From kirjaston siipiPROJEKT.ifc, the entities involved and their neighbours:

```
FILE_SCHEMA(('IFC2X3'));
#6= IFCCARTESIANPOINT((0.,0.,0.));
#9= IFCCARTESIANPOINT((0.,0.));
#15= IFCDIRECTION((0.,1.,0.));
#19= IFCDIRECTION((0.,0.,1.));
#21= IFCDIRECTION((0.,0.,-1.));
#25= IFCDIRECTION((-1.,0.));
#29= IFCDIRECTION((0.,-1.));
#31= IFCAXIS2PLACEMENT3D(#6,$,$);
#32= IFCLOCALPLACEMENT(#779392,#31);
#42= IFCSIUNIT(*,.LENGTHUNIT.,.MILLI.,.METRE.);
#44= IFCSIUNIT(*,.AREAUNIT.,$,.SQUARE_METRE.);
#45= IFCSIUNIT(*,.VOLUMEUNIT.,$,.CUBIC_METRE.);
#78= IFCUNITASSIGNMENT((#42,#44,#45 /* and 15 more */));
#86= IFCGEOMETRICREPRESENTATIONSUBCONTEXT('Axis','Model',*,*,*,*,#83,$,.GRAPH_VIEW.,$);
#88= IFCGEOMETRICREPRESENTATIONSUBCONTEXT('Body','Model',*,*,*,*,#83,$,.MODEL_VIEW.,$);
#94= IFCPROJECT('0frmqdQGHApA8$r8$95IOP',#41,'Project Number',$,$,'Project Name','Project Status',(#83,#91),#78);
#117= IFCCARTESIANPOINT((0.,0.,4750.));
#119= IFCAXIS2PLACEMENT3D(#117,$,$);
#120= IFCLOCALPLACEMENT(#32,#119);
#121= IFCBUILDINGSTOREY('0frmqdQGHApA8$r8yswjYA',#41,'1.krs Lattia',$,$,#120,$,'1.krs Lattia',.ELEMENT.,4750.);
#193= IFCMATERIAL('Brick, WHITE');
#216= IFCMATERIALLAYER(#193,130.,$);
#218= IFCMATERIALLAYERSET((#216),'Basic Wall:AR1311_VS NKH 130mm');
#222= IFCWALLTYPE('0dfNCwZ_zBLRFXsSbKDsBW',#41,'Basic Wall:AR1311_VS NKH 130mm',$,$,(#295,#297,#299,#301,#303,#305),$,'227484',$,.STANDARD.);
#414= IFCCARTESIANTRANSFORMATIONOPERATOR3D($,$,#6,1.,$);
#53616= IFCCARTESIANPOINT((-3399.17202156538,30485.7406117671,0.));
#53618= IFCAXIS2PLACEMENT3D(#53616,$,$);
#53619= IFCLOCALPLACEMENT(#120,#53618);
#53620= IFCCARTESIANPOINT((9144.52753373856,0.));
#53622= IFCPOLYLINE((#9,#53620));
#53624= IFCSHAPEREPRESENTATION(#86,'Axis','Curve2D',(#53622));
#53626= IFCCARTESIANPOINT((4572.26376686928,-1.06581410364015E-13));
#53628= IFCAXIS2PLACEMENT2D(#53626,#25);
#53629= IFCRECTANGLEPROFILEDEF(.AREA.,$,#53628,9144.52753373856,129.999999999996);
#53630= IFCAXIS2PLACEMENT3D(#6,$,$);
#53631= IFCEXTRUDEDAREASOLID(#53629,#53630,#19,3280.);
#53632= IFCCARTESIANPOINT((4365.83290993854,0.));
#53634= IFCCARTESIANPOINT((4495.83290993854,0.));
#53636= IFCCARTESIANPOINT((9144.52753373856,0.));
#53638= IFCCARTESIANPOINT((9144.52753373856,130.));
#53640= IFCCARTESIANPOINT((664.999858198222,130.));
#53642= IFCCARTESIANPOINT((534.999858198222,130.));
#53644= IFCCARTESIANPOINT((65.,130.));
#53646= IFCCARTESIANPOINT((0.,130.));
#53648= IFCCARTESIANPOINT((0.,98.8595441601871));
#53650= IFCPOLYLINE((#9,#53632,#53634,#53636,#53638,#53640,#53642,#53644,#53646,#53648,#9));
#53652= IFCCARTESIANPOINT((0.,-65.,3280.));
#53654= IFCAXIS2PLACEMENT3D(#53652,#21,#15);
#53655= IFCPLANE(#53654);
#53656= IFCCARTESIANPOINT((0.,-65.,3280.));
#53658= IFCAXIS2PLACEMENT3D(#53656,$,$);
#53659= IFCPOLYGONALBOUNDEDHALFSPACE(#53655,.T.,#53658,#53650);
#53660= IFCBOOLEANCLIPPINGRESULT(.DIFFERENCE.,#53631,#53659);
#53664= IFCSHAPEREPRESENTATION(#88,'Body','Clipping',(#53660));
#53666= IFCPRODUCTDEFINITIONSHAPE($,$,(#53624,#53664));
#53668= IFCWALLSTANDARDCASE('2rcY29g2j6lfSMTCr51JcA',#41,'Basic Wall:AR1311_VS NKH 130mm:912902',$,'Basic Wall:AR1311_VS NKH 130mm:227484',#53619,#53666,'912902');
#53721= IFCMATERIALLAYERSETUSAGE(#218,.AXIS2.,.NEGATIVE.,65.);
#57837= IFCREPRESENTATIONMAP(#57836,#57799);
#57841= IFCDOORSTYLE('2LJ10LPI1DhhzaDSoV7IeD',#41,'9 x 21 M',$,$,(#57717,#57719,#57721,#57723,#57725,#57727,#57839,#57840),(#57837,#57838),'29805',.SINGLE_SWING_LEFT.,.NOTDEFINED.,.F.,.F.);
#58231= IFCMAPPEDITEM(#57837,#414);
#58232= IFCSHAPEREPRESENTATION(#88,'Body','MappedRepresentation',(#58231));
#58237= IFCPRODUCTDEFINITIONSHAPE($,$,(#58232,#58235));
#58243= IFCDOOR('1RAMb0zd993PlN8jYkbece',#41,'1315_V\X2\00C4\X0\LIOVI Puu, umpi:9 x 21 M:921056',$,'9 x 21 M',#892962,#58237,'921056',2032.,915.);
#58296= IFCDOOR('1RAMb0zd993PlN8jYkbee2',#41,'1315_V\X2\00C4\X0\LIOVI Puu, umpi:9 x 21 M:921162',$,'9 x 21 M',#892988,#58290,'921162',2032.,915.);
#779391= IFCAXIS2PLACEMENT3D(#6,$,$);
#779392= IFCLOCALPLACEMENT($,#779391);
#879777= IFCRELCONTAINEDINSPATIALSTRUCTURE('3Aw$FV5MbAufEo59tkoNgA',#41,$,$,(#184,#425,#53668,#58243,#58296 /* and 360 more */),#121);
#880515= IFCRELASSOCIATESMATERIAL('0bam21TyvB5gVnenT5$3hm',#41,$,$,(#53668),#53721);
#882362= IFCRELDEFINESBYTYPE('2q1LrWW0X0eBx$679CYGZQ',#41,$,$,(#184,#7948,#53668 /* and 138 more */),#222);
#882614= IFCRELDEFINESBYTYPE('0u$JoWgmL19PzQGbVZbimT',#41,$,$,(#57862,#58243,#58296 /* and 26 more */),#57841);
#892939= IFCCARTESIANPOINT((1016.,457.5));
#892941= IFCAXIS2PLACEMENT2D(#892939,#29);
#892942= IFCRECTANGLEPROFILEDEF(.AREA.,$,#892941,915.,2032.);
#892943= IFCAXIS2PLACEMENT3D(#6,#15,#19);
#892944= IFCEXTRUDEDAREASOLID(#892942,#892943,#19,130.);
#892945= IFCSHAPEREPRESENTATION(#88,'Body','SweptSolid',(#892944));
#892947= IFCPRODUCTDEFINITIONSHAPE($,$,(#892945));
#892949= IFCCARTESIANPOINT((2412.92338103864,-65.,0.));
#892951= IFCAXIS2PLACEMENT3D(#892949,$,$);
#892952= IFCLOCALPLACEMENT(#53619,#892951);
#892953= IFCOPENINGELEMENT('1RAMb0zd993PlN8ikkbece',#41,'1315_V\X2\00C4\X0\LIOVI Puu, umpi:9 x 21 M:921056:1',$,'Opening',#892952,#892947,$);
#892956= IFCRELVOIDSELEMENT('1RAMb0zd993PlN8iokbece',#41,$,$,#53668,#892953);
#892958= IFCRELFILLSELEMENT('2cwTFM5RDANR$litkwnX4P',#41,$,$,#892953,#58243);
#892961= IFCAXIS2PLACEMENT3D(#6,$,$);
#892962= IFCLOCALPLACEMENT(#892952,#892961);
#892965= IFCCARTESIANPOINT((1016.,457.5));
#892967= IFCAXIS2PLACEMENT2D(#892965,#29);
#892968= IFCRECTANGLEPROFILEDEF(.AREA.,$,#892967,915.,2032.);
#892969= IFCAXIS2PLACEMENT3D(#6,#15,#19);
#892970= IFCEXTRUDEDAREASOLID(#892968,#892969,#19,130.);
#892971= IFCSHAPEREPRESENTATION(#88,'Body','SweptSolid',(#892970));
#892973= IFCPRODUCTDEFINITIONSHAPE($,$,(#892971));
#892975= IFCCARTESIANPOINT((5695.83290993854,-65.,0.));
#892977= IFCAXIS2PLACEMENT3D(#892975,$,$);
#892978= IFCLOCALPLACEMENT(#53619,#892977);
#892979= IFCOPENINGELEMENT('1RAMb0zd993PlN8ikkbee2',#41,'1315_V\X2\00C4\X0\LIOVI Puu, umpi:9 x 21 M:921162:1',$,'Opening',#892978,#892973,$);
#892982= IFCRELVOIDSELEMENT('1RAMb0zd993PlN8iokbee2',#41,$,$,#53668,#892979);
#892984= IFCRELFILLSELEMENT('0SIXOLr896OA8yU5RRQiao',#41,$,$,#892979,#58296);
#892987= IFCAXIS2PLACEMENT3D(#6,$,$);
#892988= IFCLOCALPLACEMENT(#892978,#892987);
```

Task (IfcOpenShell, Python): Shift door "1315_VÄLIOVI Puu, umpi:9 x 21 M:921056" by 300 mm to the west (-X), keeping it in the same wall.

```python
import ifcopenshell
import ifcopenshell.api.geometry
import ifcopenshell.util.placement

model = ifcopenshell.open("kirjaston siipiPROJEKT.ifc")

door = model.by_guid("1RAMb0zd993PlN8jYkbece")
opening = door.FillsVoids[0].RelatingOpeningElement
wall = opening.VoidsElements[0].RelatingBuildingElement

wall_matrix = ifcopenshell.util.placement.get_local_placement(wall.ObjectPlacement)
shift = wall_matrix[:3, 0] * -300.0
before = ifcopenshell.util.placement.get_local_placement(door.ObjectPlacement)[:3, 3].copy()

# The door is placed relative to its opening, so it follows when the opening moves.
matrix = ifcopenshell.util.placement.get_local_placement(opening.ObjectPlacement)
matrix[:3, 3] += shift
ifcopenshell.api.geometry.edit_object_placement(
    model, product=opening, matrix=matrix, is_si=False, should_transform_children=True
)

after = ifcopenshell.util.placement.get_local_placement(door.ObjectPlacement)[:3, 3]
print("door moved by", (after - before).round(3) + 0.0)

model.write("kirjaston siipiPROJEKT_v2.ifc")
```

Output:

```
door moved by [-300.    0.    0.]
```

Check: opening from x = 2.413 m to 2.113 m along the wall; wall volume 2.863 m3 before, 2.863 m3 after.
